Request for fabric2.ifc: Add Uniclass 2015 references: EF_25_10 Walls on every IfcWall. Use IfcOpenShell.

First a look at what the model holds.

```python
import ifcopenshell

model = ifcopenshell.open("fabric2.ifc")
print(model.schema)
print("classifications:", [c.Name for c in model.by_type("IfcClassification")])
for ifc_class in ("IfcDoor", "IfcRoof", "IfcStair", "IfcWall", "IfcWindow"):
    print(ifc_class, len(model.by_type(ifc_class)))
```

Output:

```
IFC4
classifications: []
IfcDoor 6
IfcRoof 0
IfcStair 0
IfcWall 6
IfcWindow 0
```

```python
import ifcopenshell
import ifcopenshell.api.classification

model = ifcopenshell.open("fabric2.ifc")

system = ifcopenshell.api.classification.add_classification(model, classification="Uniclass 2015")

codes = {
    "IfcWall": ("EF_25_10", "Walls"),
}
for ifc_class, (code, name) in codes.items():
    products = model.by_type(ifc_class)
    ifcopenshell.api.classification.add_reference(
        model, products=products, classification=system, identification=code, name=name
    )
    print(code, len(products))

model.write("fabric2_v2.ifc")
```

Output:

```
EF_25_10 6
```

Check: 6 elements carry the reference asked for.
